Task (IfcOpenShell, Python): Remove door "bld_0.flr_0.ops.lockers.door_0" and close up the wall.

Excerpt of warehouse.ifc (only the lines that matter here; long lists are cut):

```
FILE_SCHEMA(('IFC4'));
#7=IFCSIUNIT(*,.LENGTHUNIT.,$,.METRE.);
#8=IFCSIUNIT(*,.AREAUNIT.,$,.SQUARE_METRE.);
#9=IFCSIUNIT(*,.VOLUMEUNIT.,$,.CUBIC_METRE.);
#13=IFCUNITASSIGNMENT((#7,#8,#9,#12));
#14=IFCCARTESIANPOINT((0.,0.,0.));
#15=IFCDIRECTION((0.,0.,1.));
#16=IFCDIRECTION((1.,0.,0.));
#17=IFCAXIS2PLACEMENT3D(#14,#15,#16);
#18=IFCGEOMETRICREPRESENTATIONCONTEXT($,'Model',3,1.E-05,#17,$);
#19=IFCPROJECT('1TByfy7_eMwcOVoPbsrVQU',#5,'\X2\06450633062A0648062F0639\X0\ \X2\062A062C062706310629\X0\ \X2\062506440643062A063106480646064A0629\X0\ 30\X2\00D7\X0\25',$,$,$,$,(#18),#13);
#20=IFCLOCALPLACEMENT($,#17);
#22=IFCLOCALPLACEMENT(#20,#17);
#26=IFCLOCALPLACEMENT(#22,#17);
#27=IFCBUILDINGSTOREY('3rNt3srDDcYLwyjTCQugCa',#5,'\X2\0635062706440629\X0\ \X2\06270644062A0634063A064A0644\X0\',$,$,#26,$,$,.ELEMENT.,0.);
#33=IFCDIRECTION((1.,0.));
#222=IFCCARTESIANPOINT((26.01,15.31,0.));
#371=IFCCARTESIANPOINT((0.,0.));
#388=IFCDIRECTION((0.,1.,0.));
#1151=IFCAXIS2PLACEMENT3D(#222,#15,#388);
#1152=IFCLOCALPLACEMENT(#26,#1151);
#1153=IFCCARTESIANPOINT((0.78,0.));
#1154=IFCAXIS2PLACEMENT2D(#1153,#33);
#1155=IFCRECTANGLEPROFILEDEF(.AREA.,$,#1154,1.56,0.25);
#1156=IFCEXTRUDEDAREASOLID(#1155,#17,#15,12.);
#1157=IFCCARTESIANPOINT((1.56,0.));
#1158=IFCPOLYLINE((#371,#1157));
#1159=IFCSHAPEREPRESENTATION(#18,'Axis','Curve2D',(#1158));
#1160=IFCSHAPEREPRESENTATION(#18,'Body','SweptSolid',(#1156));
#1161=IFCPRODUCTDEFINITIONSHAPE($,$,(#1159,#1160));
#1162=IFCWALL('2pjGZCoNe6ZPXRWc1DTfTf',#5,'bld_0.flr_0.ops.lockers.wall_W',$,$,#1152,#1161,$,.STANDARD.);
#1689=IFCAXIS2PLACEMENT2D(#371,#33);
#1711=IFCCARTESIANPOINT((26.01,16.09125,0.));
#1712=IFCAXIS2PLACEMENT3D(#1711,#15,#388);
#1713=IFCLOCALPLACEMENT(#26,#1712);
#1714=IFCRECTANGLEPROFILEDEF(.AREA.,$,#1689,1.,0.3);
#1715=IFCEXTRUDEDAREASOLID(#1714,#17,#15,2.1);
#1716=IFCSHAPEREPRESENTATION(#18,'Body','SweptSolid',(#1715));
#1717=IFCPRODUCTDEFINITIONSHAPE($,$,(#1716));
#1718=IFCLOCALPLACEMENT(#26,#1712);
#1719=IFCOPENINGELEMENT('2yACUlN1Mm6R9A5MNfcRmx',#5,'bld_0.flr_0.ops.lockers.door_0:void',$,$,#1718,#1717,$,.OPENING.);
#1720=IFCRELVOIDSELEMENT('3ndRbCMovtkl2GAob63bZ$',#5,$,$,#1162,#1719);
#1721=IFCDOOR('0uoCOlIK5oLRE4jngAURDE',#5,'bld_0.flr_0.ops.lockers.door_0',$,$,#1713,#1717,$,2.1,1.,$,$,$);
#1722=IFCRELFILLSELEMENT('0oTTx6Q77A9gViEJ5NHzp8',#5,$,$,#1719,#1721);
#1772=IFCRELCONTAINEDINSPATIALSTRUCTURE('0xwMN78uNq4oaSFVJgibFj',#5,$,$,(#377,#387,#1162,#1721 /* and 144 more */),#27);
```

```python
import ifcopenshell
import ifcopenshell.api.feature
import ifcopenshell.api.root
import ifcopenshell.geom
import ifcopenshell.util.shape

model = ifcopenshell.open("warehouse.ifc")
settings = ifcopenshell.geom.settings()


def volume(element):
    """Net volume in cubic metres, openings subtracted."""
    shape = ifcopenshell.geom.create_shape(settings, element)
    return ifcopenshell.util.shape.get_volume(shape.geometry)


door = model.by_guid("0uoCOlIK5oLRE4jngAURDE")
opening = door.FillsVoids[0].RelatingOpeningElement
wall = opening.VoidsElements[0].RelatingBuildingElement
before = volume(wall)

ifcopenshell.api.root.remove_product(model, product=door)
ifcopenshell.api.feature.remove_feature(model, feature=opening)

after = volume(wall)

print(f"wall volume {before:.3f} -> {after:.3f} m3")

model.write("warehouse_v2.ifc")
```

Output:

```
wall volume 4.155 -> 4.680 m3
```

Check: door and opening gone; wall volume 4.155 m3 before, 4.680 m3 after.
